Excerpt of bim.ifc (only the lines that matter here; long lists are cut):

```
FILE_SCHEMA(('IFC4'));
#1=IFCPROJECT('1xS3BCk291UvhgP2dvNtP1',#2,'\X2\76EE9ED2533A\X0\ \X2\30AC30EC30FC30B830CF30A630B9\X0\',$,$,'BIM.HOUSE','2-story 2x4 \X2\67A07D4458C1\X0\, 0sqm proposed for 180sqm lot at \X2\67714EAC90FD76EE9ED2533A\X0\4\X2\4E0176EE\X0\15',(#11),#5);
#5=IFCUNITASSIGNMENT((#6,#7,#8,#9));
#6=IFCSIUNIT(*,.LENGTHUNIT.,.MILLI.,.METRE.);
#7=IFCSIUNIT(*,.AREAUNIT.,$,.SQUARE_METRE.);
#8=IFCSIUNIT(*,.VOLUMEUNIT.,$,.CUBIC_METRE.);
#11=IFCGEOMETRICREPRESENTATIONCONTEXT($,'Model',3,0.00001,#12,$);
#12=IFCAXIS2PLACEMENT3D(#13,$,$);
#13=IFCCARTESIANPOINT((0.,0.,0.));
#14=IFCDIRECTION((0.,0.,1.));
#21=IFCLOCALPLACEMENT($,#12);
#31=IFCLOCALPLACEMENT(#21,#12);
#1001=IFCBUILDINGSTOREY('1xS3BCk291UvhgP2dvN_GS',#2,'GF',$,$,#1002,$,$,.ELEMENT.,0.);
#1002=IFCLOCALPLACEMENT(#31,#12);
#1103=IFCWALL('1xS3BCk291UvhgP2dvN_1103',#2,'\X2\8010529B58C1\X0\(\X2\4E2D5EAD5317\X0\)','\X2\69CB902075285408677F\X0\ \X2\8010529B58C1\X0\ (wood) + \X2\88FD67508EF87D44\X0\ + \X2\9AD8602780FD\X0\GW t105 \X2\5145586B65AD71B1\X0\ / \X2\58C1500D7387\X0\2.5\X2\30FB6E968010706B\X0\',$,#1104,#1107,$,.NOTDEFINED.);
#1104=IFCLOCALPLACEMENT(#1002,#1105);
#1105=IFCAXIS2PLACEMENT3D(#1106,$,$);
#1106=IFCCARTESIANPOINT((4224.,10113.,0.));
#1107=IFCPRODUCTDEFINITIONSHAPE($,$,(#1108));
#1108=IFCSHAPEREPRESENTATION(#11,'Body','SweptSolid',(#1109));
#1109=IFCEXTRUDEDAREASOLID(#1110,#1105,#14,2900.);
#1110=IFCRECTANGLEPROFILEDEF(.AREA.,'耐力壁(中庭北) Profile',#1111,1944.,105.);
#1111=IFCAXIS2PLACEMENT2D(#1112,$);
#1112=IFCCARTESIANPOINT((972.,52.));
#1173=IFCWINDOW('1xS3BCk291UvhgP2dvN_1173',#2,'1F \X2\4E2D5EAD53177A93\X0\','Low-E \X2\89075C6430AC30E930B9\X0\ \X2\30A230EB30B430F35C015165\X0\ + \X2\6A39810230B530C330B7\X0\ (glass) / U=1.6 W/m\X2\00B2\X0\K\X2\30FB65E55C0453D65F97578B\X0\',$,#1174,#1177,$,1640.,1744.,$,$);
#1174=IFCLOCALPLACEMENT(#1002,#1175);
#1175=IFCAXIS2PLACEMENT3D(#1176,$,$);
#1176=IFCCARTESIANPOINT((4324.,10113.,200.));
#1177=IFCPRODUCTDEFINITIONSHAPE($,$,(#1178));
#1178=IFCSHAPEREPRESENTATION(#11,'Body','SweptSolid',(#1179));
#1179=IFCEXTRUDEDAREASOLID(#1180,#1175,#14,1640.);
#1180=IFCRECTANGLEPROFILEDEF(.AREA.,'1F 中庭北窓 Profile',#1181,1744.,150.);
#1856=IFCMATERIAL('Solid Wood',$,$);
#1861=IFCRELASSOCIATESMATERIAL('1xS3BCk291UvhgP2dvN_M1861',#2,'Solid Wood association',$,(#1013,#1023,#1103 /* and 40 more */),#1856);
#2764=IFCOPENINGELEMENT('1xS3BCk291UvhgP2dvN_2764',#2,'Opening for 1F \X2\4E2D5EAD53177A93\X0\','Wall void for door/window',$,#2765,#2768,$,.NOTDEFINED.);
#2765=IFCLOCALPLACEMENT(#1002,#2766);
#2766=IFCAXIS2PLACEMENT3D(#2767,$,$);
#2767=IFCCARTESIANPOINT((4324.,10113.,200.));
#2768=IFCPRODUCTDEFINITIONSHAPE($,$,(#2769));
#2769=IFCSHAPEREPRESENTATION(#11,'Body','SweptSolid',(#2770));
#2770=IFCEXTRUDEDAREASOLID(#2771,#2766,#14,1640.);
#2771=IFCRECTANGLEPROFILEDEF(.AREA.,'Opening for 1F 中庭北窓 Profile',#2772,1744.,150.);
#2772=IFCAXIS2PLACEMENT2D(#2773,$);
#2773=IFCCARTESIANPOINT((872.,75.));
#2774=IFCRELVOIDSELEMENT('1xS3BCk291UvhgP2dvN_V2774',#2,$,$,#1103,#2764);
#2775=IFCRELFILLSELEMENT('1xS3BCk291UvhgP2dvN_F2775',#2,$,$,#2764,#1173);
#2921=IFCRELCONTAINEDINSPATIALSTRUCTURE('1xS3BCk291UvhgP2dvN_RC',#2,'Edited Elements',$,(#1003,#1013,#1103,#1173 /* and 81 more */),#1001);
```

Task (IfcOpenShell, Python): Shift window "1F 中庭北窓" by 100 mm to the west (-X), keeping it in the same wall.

```python
import ifcopenshell
import ifcopenshell.api.geometry
import ifcopenshell.util.placement

model = ifcopenshell.open("bim.ifc")

window = model.by_id(1173)
opening = window.FillsVoids[0].RelatingOpeningElement
wall = opening.VoidsElements[0].RelatingBuildingElement

wall_matrix = ifcopenshell.util.placement.get_local_placement(wall.ObjectPlacement)
shift = wall_matrix[:3, 0] * -100.0
before = ifcopenshell.util.placement.get_local_placement(window.ObjectPlacement)[:3, 3].copy()

# The window is not placed relative to its opening, so move both.
for product in (opening, window):
    matrix = ifcopenshell.util.placement.get_local_placement(product.ObjectPlacement)
    matrix[:3, 3] += shift
    ifcopenshell.api.geometry.edit_object_placement(model, product=product, matrix=matrix, is_si=False)

after = ifcopenshell.util.placement.get_local_placement(window.ObjectPlacement)[:3, 3]
print("window moved by", (after - before).round(3) + 0.0)

model.write("bim_v2.ifc")
```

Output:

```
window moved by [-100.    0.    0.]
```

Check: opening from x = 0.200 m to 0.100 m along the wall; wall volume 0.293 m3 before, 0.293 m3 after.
